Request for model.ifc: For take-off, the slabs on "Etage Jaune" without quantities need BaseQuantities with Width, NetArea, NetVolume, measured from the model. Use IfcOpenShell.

First a look at what the model holds.

```python
import ifcopenshell
import ifcopenshell.util.element
import ifcopenshell.util.unit

model = ifcopenshell.open("model.ifc")
print(model.schema)
for unit_type in ("LENGTHUNIT", "AREAUNIT", "VOLUMEUNIT"):
    print(unit_type, ifcopenshell.util.unit.calculate_unit_scale(model, unit_type))
storey = next(s for s in model.by_type("IfcBuildingStorey") if s.Name == "Etage Jaune")
slabs = [e for e in ifcopenshell.util.element.get_decomposition(storey) if e.is_a("IfcSlab")]
for e in sorted(slabs, key=lambda e: e.id()):
    print(e.id(), e.is_a(), e.Name, list(ifcopenshell.util.element.get_psets(e, qtos_only=True)), sep=" | ")
```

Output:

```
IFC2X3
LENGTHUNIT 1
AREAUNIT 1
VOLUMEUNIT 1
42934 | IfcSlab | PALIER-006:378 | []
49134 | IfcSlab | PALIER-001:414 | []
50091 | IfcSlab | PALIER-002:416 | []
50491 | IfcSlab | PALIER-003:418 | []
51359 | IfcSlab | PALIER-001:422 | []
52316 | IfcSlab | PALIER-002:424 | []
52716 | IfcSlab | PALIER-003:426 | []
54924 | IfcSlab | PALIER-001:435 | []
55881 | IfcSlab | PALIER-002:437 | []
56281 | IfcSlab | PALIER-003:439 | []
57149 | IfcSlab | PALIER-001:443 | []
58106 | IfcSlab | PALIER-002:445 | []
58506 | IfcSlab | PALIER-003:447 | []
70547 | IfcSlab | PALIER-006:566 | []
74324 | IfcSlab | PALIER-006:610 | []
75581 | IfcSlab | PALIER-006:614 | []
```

```python
import ifcopenshell
import ifcopenshell.api.pset
import ifcopenshell.geom
import ifcopenshell.util.element
import ifcopenshell.util.shape
import ifcopenshell.util.unit

model = ifcopenshell.open("model.ifc")
unit_scale = ifcopenshell.util.unit.calculate_unit_scale(model)
area_scale = ifcopenshell.util.unit.calculate_unit_scale(model, "AREAUNIT")
volume_scale = ifcopenshell.util.unit.calculate_unit_scale(model, "VOLUMEUNIT")
settings = ifcopenshell.geom.settings()

storey = next(s for s in model.by_type("IfcBuildingStorey") if s.Name == "Etage Jaune")
slabs = [e for e in ifcopenshell.util.element.get_decomposition(storey) if e.is_a("IfcSlab")]

for e in sorted(slabs, key=lambda e: e.id()):
    if ifcopenshell.util.element.get_psets(e, qtos_only=True, should_inherit=False):
        continue
    # Geometry comes back in metres, in the element's own axes.
    shape = ifcopenshell.geom.create_shape(settings, e)
    values = {
        "Width": ifcopenshell.util.shape.get_z(shape.geometry) / unit_scale,
        "NetArea": ifcopenshell.util.shape.get_footprint_area(shape.geometry) / area_scale,
        "NetVolume": ifcopenshell.util.shape.get_volume(shape.geometry) / volume_scale,
    }
    qto = ifcopenshell.api.pset.add_qto(model, product=e, name="BaseQuantities")
    ifcopenshell.api.pset.edit_qto(model, qto=qto, properties=values)
    print(e.id(), {k: round(v, 3) for k, v in values.items()})

model.write("model_edited.ifc")
```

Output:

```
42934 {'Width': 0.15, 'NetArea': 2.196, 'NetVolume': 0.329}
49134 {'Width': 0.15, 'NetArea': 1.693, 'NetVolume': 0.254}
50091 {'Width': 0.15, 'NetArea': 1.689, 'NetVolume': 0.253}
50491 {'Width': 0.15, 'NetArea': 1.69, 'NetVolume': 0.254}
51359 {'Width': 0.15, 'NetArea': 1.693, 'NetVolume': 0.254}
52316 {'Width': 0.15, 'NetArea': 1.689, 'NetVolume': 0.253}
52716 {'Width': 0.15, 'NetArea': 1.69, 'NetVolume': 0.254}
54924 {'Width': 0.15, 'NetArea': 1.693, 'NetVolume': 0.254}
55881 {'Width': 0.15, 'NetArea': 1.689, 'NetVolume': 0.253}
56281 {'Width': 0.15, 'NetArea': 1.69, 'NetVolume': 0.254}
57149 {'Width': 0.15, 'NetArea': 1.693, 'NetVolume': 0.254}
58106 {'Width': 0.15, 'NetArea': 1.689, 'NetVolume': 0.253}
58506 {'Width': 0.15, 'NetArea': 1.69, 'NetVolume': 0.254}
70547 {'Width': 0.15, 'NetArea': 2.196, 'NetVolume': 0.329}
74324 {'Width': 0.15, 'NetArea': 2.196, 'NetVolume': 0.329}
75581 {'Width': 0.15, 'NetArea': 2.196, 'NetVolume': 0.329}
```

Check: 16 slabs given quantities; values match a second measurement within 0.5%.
